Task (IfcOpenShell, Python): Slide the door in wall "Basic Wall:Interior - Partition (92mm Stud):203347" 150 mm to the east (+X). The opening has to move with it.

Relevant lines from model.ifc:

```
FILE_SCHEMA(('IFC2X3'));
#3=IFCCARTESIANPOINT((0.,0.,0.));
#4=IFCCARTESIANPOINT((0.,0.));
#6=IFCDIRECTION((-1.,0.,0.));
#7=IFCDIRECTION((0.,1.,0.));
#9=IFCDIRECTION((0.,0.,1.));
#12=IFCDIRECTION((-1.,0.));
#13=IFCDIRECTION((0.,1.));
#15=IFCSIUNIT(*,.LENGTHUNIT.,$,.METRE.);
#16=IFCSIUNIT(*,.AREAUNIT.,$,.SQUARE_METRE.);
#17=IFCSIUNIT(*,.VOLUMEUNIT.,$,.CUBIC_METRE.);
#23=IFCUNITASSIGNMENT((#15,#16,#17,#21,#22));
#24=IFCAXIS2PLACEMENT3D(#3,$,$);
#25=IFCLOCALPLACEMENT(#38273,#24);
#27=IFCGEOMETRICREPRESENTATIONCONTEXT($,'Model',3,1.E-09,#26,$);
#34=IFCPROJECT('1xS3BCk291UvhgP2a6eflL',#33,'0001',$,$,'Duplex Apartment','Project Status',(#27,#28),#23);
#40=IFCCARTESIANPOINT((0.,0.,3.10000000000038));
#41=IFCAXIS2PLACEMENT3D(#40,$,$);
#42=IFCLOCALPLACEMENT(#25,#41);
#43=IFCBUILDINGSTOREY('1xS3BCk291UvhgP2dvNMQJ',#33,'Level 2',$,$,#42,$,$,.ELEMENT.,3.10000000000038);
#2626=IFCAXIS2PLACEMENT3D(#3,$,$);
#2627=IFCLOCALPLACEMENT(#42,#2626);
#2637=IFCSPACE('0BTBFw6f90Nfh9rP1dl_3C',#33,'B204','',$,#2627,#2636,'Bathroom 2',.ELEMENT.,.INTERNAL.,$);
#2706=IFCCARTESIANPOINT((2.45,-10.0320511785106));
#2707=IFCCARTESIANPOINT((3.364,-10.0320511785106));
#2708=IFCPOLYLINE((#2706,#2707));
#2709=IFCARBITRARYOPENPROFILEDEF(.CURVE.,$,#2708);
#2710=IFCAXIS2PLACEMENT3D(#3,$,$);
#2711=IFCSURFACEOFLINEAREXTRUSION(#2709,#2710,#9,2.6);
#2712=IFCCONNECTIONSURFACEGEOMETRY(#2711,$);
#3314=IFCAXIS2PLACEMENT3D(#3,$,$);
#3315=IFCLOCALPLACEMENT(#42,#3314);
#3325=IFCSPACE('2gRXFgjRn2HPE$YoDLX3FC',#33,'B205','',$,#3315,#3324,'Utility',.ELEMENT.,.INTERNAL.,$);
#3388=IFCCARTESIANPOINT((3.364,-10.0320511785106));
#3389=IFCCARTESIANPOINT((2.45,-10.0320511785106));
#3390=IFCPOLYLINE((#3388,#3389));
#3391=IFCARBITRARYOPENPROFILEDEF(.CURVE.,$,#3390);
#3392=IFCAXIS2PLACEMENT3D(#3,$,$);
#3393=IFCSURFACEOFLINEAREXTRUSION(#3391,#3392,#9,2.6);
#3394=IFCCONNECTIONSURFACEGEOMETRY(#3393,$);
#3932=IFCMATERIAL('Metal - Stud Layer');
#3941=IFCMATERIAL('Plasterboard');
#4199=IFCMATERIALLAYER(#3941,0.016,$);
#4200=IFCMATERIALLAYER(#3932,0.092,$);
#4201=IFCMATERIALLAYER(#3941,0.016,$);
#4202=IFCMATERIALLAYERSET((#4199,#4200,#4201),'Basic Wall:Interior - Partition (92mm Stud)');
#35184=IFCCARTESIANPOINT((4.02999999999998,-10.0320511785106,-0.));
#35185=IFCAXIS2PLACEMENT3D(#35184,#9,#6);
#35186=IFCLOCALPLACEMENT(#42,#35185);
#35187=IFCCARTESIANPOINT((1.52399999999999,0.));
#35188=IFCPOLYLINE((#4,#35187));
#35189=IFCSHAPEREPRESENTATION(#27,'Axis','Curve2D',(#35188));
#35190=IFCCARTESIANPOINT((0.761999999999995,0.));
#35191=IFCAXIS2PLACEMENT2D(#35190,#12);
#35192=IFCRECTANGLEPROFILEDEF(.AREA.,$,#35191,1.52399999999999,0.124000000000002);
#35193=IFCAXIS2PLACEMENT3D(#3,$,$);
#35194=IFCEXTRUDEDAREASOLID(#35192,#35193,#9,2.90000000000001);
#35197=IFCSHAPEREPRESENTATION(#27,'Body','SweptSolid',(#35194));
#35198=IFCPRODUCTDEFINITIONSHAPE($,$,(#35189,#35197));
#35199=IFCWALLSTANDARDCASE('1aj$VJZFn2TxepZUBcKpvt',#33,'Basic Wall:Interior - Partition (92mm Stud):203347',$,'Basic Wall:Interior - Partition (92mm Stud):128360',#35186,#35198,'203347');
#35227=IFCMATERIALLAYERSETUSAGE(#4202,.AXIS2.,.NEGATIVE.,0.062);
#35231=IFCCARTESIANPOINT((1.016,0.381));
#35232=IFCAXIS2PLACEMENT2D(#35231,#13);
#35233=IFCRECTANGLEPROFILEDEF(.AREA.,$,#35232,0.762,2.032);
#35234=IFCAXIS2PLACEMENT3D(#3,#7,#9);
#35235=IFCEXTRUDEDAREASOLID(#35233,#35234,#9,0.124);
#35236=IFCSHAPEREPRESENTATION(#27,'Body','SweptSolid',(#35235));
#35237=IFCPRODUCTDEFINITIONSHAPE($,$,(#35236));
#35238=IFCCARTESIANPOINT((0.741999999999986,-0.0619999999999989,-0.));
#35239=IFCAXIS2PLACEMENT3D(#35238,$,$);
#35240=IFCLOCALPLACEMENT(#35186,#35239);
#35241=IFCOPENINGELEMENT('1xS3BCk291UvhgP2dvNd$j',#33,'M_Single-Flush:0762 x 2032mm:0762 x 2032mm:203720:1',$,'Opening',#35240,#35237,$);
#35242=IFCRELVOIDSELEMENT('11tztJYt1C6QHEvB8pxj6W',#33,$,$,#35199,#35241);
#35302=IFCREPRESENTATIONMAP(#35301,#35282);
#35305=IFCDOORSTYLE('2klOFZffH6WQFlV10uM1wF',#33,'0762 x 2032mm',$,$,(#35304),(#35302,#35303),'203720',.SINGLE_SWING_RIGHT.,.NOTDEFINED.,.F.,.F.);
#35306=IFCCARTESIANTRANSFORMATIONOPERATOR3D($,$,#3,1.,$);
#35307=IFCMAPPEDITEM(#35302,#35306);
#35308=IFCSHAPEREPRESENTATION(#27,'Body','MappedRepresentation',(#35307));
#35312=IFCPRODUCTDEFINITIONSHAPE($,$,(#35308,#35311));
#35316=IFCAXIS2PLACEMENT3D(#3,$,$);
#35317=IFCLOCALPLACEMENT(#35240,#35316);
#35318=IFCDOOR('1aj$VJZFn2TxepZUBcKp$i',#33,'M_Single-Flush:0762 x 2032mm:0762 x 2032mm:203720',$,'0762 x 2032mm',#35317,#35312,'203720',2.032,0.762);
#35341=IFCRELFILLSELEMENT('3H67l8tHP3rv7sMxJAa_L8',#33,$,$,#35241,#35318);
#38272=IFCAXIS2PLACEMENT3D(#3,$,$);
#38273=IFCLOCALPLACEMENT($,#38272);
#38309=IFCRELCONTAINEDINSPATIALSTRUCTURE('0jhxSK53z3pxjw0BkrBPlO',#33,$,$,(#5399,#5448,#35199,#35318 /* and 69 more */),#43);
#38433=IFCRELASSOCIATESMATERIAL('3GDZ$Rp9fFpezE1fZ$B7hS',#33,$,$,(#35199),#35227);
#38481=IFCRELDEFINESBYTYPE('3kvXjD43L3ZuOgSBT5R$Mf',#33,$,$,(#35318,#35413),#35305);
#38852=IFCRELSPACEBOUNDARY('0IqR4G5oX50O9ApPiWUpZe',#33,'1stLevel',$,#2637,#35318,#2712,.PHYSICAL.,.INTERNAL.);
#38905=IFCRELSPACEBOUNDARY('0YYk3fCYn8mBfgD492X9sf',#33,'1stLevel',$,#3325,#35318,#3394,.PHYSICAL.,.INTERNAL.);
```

```python
import numpy as np
import ifcopenshell
import ifcopenshell.api.geometry
import ifcopenshell.util.placement
import ifcopenshell.util.unit

model = ifcopenshell.open("model.ifc")
unit_scale = ifcopenshell.util.unit.calculate_unit_scale(model)

door = model.by_guid("1aj$VJZFn2TxepZUBcKp$i")
opening = door.FillsVoids[0].RelatingOpeningElement
wall = opening.VoidsElements[0].RelatingBuildingElement

wall_matrix = ifcopenshell.util.placement.get_local_placement(wall.ObjectPlacement)
shift = wall_matrix[:3, 0] * -0.15 / unit_scale
before = ifcopenshell.util.placement.get_local_placement(door.ObjectPlacement)[:3, 3].copy()

# The door is placed relative to its opening, so it follows when the opening moves.
matrix = ifcopenshell.util.placement.get_local_placement(opening.ObjectPlacement)
matrix[:3, 3] += shift
ifcopenshell.api.geometry.edit_object_placement(
    model, product=opening, matrix=matrix, is_si=False, should_transform_children=True
)

# Space boundary surfaces are stored in each space's coordinates; move them too.
for rel in door.ProvidesBoundaries:
    if not rel.ConnectionGeometry:
        continue
    surface = rel.ConnectionGeometry.SurfaceOnRelatingElement
    space_matrix = ifcopenshell.util.placement.get_local_placement(rel.RelatingSpace.ObjectPlacement)
    point = np.array(surface.Position.Location.Coordinates) + space_matrix[:3, :3].T @ shift
    surface.Position = model.createIfcAxis2Placement3D(
        model.createIfcCartesianPoint(point.tolist()), surface.Position.Axis, surface.Position.RefDirection
    )

after = ifcopenshell.util.placement.get_local_placement(door.ObjectPlacement)[:3, 3]
print("door moved by", (after - before).round(3) + 0.0)

model.write("model_updated.ifc")
```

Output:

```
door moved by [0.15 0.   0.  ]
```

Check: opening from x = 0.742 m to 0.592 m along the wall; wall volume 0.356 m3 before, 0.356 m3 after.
